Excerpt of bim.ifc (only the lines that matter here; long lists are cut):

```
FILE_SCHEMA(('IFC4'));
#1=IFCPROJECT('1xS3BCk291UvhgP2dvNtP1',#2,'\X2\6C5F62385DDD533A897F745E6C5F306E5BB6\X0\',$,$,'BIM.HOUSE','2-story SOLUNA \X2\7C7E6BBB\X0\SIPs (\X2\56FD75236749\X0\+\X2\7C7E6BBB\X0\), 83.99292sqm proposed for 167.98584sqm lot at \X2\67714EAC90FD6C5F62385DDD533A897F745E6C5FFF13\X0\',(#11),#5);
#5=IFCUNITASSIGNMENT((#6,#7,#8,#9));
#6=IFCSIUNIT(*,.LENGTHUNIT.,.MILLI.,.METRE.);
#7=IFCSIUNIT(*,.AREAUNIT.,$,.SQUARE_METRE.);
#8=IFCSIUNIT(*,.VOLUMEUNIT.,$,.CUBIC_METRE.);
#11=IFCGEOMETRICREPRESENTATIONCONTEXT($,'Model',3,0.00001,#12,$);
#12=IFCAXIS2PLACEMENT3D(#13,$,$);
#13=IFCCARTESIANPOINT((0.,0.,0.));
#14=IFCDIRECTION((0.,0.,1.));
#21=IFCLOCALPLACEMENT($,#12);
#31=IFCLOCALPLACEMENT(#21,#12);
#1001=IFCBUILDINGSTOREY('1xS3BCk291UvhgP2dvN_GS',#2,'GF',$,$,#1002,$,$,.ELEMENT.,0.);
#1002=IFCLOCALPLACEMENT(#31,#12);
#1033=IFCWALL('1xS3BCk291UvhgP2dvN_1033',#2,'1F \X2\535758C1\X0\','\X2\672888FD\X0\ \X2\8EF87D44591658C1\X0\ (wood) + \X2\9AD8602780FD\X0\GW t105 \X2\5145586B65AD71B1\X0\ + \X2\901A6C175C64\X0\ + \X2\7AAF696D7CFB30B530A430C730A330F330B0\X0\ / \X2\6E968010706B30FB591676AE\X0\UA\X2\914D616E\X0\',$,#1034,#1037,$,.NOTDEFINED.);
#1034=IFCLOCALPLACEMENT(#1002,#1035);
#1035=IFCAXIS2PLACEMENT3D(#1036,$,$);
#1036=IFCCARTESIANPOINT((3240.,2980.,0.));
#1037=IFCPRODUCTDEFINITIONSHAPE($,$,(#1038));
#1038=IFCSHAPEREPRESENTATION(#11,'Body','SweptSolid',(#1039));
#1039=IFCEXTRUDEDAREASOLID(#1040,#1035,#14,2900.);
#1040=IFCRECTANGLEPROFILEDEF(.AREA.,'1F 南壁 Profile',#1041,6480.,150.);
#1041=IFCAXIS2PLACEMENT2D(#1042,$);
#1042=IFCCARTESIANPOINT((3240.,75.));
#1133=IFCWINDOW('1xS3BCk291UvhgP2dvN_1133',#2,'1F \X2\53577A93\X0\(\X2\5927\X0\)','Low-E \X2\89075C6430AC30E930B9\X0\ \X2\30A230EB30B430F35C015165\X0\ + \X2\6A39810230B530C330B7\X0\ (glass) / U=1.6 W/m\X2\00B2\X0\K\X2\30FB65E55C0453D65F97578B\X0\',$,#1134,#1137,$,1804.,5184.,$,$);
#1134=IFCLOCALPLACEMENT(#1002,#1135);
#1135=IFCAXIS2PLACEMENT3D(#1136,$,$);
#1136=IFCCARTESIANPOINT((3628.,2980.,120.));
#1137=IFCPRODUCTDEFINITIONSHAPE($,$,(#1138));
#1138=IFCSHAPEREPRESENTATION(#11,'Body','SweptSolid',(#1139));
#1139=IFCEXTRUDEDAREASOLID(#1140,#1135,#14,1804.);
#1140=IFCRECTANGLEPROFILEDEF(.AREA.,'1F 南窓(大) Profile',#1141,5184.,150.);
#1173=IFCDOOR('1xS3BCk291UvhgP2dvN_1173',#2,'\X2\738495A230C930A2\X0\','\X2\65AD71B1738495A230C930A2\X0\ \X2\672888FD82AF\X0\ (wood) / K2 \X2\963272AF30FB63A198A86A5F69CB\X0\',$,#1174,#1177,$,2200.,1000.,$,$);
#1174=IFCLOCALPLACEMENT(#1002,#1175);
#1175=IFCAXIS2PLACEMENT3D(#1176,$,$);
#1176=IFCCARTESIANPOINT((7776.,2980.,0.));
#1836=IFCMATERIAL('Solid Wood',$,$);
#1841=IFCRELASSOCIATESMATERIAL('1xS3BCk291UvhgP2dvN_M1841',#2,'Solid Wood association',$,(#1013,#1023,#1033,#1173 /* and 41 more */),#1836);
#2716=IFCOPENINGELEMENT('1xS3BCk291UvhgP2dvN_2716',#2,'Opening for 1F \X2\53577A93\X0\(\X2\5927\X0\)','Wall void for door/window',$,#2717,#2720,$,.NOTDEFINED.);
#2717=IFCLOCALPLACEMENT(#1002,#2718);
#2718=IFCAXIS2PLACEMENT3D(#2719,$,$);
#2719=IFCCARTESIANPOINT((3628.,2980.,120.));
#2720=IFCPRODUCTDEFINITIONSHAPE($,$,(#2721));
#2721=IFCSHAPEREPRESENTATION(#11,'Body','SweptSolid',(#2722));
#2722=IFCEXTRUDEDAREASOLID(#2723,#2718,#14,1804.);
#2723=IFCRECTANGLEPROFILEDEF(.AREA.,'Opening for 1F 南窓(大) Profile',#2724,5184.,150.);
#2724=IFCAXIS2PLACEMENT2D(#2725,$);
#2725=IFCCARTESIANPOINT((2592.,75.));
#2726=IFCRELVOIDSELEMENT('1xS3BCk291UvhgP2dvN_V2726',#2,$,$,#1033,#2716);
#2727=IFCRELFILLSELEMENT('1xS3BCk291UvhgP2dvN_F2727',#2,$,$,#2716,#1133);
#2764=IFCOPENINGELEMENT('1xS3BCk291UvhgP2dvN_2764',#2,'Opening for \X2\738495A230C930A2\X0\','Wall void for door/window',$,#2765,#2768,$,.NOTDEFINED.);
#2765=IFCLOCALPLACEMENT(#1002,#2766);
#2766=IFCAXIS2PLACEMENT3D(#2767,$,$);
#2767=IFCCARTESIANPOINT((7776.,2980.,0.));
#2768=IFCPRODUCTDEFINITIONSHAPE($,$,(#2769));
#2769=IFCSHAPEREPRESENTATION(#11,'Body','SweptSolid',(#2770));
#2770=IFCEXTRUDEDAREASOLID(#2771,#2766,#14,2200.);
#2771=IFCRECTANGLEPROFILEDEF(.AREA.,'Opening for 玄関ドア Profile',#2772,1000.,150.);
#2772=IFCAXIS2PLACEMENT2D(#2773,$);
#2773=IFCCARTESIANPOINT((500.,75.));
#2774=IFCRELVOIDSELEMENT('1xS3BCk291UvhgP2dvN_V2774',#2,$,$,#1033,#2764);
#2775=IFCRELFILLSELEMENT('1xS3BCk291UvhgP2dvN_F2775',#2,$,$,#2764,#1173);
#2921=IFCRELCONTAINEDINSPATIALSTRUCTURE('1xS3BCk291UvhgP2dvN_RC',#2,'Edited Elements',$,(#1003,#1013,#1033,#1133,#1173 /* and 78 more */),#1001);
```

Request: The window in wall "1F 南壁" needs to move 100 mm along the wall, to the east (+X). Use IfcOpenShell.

```python
import ifcopenshell
import ifcopenshell.api.geometry
import ifcopenshell.util.placement
import ifcopenshell.util.unit

model = ifcopenshell.open("bim.ifc")
unit_scale = ifcopenshell.util.unit.calculate_unit_scale(model)

window = model.by_guid("1xS3BCk291UvhgP2dvN_1133")
opening = window.FillsVoids[0].RelatingOpeningElement
wall = opening.VoidsElements[0].RelatingBuildingElement

wall_matrix = ifcopenshell.util.placement.get_local_placement(wall.ObjectPlacement)
shift = wall_matrix[:3, 0] * 0.1 / unit_scale
before = ifcopenshell.util.placement.get_local_placement(window.ObjectPlacement)[:3, 3].copy()

# The window is not placed relative to its opening, so move both.
for product in (opening, window):
    matrix = ifcopenshell.util.placement.get_local_placement(product.ObjectPlacement)
    matrix[:3, 3] += shift
    ifcopenshell.api.geometry.edit_object_placement(model, product=product, matrix=matrix, is_si=False)

after = ifcopenshell.util.placement.get_local_placement(window.ObjectPlacement)[:3, 3]
print("window moved by", (after - before).round(3) + 0.0)

model.write("bim_edited.ifc")
```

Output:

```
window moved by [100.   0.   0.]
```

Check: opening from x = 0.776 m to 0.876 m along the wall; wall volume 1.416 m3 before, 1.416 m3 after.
